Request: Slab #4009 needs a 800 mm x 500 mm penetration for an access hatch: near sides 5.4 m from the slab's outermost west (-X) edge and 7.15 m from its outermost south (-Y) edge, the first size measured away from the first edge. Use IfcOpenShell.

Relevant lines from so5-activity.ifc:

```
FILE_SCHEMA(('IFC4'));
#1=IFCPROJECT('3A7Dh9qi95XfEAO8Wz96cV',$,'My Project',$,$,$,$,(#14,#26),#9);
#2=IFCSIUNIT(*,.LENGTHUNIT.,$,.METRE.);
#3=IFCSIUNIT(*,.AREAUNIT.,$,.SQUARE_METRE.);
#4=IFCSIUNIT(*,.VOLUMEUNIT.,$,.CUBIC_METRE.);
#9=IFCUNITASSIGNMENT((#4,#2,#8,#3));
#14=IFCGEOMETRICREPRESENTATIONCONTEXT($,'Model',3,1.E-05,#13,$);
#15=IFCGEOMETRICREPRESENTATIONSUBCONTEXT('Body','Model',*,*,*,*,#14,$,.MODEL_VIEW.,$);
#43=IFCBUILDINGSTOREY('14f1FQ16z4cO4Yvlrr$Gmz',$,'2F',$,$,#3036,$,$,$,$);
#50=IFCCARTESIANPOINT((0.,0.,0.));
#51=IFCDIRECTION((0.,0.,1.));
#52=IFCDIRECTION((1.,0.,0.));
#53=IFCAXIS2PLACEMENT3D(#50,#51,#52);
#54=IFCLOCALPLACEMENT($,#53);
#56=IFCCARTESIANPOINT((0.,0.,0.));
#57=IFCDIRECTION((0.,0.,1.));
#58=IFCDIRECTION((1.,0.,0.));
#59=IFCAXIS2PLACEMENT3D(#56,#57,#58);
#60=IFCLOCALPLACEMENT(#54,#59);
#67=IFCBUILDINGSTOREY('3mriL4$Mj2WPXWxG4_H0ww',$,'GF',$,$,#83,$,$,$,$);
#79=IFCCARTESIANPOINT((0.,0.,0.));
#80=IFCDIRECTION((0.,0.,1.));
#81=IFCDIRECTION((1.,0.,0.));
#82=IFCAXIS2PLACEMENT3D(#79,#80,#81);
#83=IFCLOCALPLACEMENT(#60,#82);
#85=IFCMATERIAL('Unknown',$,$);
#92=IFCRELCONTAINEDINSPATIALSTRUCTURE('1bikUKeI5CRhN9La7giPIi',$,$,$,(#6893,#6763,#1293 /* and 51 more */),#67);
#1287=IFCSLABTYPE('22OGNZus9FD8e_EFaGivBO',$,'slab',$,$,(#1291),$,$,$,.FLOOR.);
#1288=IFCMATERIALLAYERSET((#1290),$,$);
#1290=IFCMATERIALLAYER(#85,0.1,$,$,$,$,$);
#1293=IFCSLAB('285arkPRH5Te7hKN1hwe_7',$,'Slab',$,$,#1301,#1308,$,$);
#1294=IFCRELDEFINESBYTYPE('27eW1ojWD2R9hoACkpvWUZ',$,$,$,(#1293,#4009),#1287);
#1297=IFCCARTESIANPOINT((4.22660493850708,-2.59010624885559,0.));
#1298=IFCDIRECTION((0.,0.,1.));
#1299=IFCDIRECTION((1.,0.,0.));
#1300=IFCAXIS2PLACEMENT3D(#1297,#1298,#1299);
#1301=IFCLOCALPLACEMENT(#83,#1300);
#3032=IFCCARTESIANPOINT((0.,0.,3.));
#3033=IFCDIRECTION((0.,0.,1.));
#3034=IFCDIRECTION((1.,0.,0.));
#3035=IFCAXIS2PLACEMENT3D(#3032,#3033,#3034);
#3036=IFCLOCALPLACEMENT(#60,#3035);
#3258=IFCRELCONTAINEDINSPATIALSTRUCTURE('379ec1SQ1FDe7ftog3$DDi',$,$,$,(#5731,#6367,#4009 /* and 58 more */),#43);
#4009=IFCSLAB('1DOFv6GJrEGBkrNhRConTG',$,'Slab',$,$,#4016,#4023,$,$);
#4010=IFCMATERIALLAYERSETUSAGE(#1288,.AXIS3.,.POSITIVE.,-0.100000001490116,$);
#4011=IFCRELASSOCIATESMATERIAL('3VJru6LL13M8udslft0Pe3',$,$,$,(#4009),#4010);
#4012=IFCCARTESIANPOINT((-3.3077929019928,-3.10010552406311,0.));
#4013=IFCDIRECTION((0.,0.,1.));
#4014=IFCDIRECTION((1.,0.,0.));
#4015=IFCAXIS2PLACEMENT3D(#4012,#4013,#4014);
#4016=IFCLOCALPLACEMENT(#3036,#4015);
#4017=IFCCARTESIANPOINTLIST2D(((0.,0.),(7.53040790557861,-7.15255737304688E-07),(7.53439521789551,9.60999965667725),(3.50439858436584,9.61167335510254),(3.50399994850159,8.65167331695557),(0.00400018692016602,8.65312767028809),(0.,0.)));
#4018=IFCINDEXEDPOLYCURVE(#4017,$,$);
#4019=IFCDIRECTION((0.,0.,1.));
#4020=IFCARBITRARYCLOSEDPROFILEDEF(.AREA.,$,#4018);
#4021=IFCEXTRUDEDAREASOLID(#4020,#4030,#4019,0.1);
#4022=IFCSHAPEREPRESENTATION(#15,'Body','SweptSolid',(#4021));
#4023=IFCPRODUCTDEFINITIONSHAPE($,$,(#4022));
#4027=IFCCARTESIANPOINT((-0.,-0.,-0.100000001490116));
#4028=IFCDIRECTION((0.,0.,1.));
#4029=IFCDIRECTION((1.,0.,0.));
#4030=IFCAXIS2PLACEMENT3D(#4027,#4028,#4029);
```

```python
import numpy as np
import ifcopenshell
import ifcopenshell.api.feature
import ifcopenshell.api.geometry
import ifcopenshell.api.root
import ifcopenshell.geom
import ifcopenshell.util.placement
import ifcopenshell.util.representation
import ifcopenshell.util.shape
import ifcopenshell.util.unit

model = ifcopenshell.open("so5-activity.ifc")
unit_scale = ifcopenshell.util.unit.calculate_unit_scale(model)
settings = ifcopenshell.geom.settings()


def volume(element):
    """Net volume in cubic metres, openings subtracted."""
    shape = ifcopenshell.geom.create_shape(settings, element)
    return ifcopenshell.util.shape.get_volume(shape.geometry)


slab = model.by_guid("1DOFv6GJrEGBkrNhRConTG")
before = volume(slab)

# Extent in the slab's own axes, in metres. The edges named are its -X and -Y sides.
slab_shape = ifcopenshell.geom.create_shape(settings, slab)
vertices = ifcopenshell.util.shape.get_vertices(slab_shape.geometry)
x_min, y_min, bottom = vertices.min(axis=0)
top = vertices[:, 2].max()

opening = ifcopenshell.api.root.create_entity(model, ifc_class="IfcOpeningElement", name="Access hatch opening", predefined_type="OPENING")
context = ifcopenshell.util.representation.get_context(model, "Model", "Body", "MODEL_VIEW")
width, depth = 0.8, 0.5
outline = [(0.0, 0.0), (width, 0.0), (width, depth), (0.0, depth), (0.0, 0.0)]
# Overshoot both faces by 50 mm so the cut is clean.
shape = ifcopenshell.api.geometry.add_slab_representation(
    model, context=context, depth=top - bottom + 0.1, polyline=outline
)
ifcopenshell.api.geometry.assign_representation(model, product=opening, representation=shape)

matrix = ifcopenshell.util.placement.get_local_placement(slab.ObjectPlacement)
matrix[:, 3] = matrix @ np.append(np.array([x_min + 5.4, y_min + 7.15, bottom - 0.05]) / unit_scale, 1.0)
ifcopenshell.api.geometry.edit_object_placement(model, product=opening, matrix=matrix, is_si=False)
ifcopenshell.api.feature.add_feature(model, feature=opening, element=slab)

after = volume(slab)

print(f"slab volume {before:.3f} -> {after:.3f} m3")

model.write("so5-activity-out.ifc")
```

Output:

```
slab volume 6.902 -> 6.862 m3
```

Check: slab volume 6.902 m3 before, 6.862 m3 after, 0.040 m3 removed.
